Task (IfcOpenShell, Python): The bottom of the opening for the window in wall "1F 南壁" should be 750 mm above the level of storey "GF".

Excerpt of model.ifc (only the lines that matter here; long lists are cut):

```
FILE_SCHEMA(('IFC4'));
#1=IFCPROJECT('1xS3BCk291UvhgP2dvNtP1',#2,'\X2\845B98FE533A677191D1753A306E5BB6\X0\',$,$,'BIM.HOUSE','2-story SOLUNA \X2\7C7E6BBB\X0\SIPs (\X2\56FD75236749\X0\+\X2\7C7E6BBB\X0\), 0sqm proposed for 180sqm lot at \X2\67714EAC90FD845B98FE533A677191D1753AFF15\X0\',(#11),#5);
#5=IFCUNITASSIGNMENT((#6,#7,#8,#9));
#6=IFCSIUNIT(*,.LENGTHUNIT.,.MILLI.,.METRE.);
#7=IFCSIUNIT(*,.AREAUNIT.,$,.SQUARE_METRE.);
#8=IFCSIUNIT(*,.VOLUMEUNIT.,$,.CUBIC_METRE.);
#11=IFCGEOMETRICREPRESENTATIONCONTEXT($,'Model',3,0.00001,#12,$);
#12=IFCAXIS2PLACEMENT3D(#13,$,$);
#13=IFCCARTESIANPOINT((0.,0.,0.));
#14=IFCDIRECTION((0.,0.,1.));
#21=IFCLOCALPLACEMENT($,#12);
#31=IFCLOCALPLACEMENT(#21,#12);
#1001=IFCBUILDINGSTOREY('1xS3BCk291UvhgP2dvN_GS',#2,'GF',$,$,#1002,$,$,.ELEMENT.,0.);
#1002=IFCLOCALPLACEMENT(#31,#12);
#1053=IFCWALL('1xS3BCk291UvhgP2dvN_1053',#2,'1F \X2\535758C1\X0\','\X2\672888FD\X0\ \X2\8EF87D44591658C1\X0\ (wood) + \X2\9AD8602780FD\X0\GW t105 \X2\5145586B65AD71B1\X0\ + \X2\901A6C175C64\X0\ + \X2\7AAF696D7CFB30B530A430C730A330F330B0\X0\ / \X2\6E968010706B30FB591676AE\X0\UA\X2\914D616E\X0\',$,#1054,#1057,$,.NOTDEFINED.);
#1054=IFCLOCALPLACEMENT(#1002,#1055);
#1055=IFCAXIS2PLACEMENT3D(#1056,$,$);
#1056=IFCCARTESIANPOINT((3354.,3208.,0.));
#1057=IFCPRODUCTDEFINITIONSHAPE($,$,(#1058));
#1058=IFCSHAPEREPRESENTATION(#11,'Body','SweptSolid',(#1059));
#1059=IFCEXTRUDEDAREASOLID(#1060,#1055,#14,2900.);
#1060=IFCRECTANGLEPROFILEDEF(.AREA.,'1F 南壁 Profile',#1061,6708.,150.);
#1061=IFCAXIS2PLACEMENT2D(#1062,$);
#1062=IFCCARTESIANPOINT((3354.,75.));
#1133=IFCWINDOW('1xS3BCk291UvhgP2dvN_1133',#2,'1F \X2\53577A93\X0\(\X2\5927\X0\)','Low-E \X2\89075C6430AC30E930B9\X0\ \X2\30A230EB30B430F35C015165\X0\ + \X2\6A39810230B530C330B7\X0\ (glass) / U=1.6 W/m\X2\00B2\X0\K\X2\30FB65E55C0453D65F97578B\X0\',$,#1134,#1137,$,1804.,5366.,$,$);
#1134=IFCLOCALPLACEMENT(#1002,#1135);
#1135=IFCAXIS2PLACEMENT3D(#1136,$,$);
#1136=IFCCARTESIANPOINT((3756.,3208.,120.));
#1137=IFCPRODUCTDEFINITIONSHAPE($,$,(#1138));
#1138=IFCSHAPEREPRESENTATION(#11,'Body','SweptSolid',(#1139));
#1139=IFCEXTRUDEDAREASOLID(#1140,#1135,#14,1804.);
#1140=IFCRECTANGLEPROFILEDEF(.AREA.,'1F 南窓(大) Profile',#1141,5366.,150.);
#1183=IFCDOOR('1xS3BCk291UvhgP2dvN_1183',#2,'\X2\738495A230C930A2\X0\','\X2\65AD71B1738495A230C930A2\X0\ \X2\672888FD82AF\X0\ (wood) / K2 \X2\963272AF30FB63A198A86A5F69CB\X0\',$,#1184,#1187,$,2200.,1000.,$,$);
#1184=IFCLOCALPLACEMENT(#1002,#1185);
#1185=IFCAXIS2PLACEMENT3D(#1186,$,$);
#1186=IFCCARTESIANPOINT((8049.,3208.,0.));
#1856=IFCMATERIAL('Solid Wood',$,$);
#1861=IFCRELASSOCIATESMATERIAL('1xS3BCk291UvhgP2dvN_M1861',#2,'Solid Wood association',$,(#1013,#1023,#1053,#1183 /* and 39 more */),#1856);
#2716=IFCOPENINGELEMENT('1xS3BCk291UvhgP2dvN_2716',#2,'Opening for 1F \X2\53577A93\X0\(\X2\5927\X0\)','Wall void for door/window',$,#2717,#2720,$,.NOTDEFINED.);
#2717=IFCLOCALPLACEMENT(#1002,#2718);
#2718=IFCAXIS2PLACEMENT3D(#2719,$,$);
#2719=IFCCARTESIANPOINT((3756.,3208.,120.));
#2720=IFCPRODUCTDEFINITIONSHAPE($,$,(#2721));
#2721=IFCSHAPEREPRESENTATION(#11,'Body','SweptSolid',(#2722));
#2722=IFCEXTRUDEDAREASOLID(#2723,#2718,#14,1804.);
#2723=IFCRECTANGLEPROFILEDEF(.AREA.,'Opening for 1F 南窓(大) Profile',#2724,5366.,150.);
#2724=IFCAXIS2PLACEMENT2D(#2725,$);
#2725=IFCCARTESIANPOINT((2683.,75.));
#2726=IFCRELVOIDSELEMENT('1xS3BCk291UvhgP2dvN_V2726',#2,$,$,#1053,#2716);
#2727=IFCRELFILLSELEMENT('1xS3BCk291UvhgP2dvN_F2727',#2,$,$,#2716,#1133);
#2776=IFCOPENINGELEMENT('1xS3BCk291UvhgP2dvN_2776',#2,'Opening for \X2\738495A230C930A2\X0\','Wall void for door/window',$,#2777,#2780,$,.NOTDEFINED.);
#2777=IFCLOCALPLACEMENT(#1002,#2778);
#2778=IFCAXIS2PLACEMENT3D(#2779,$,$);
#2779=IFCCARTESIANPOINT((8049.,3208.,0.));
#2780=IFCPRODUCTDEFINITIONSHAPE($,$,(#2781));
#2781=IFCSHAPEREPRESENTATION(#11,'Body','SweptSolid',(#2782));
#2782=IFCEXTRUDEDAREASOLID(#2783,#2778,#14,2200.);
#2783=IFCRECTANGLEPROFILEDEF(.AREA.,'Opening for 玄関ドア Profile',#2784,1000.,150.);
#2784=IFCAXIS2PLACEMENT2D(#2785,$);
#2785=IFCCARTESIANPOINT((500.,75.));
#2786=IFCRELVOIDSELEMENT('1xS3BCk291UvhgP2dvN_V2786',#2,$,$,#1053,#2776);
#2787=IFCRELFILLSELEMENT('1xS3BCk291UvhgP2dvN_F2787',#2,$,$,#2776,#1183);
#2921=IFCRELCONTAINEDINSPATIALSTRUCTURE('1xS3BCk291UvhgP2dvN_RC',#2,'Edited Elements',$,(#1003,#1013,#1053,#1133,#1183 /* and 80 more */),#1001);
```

```python
import numpy as np
import ifcopenshell
import ifcopenshell.api.geometry
import ifcopenshell.geom
import ifcopenshell.util.element
import ifcopenshell.util.placement
import ifcopenshell.util.shape
import ifcopenshell.util.unit

model = ifcopenshell.open("model.ifc")
unit_scale = ifcopenshell.util.unit.calculate_unit_scale(model)

window = model.by_id(1133)
opening = window.FillsVoids[0].RelatingOpeningElement
storey = ifcopenshell.util.element.get_container(window, ifc_class="IfcBuildingStorey")
level = ifcopenshell.util.placement.get_local_placement(storey.ObjectPlacement)[2, 3]

# The opening's origin need not be at the sill, so measure its lowest point.
shape = ifcopenshell.geom.create_shape(ifcopenshell.geom.settings(), opening)
bottom = ifcopenshell.util.shape.get_shape_bottom_elevation(shape, shape.geometry) / unit_scale
dz = level + 0.75 / unit_scale - bottom

shift = np.array([0.0, 0.0, dz])
# The window is not placed relative to its opening, so move both.
for product in (opening, window):
    matrix = ifcopenshell.util.placement.get_local_placement(product.ObjectPlacement)
    matrix[:3, 3] += shift
    ifcopenshell.api.geometry.edit_object_placement(model, product=product, matrix=matrix, is_si=False)

print(f"moved by {dz * unit_scale:+.3f} m")

model.write("model_rev.ifc")
```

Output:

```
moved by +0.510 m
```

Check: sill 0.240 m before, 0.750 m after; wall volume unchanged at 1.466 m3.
